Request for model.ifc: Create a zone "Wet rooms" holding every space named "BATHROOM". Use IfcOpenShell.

First a look at what the model holds.

```python
import ifcopenshell

model = ifcopenshell.open("model.ifc")
print(model.schema)
seen = {}
for space in model.by_type("IfcSpace"):
    seen[space.LongName] = seen.get(space.LongName, 0) + 1
for name, count in sorted(seen.items(), key=str):
    print(count, "x", name)
print("zones:", [z.Name for z in model.by_type("IfcZone")][:20])
```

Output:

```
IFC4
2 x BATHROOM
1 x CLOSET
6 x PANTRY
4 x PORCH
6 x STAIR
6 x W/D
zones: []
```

```python
import ifcopenshell
import ifcopenshell.api.group
import ifcopenshell.api.root

model = ifcopenshell.open("model.ifc")

names = {"BATHROOM"}
spaces = [s for s in model.by_type("IfcSpace") if s.LongName in names]

zone = ifcopenshell.api.root.create_entity(model, ifc_class="IfcZone", name="Wet rooms")
ifcopenshell.api.group.assign_group(model, products=spaces, group=zone)
print(len(spaces), "spaces in", zone.Name)

model.write("model_edited.ifc")
```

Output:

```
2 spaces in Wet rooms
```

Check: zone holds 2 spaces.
